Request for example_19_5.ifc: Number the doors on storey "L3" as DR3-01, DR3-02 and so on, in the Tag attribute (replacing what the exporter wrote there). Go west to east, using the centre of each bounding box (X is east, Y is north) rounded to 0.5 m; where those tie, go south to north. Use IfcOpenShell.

First a look at what the model holds.

```python
import ifcopenshell
import ifcopenshell.util.element
import ifcopenshell.util.placement

model = ifcopenshell.open("example_19_5.ifc")
print(model.schema)
storey = next(s for s in model.by_type("IfcBuildingStorey") if s.Name == "L3")
doors = [e for e in ifcopenshell.util.element.get_decomposition(storey) if e.is_a("IfcDoor")]
for e in sorted(doors, key=lambda e: e.id()):
    origin = ifcopenshell.util.placement.get_local_placement(e.ObjectPlacement)[:3, 3]
    print(e.id(), e.Tag, e.Name, origin.round(2) + 0.0, sep=" | ")
```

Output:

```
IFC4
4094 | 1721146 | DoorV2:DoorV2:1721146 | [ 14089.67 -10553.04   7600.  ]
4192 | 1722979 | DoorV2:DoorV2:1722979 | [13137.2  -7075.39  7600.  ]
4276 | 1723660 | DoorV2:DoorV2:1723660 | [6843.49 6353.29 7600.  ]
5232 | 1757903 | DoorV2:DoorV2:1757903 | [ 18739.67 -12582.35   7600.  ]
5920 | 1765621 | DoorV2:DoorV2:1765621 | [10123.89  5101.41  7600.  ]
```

```python
import ifcopenshell
import ifcopenshell.geom
import ifcopenshell.util.element
import ifcopenshell.util.shape

model = ifcopenshell.open("example_19_5.ifc")
settings = ifcopenshell.geom.settings()
settings.set("use-world-coords", True)


def centre(element):
    shape = ifcopenshell.geom.create_shape(settings, element)
    return ifcopenshell.util.shape.get_bbox_centroid(shape.geometry)


storey = next(s for s in model.by_type("IfcBuildingStorey") if s.Name == "L3")
doors = [e for e in ifcopenshell.util.element.get_decomposition(storey) if e.is_a("IfcDoor")]

# Insertion points can sit at a corner or the storey origin, so sort by the geometry (in metres).
centres = {e: centre(e) for e in doors}
doors.sort(key=lambda e: (round(centres[e][0] / 0.5), centres[e][1]))

for i, e in enumerate(doors, start=1):
    number = f"DR3-{i:02d}"
    e.Tag = number
    print(e.id(), number)

model.write("example_19_5_v2.ifc")
```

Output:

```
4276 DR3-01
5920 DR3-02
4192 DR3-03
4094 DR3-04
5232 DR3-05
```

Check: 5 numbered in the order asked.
